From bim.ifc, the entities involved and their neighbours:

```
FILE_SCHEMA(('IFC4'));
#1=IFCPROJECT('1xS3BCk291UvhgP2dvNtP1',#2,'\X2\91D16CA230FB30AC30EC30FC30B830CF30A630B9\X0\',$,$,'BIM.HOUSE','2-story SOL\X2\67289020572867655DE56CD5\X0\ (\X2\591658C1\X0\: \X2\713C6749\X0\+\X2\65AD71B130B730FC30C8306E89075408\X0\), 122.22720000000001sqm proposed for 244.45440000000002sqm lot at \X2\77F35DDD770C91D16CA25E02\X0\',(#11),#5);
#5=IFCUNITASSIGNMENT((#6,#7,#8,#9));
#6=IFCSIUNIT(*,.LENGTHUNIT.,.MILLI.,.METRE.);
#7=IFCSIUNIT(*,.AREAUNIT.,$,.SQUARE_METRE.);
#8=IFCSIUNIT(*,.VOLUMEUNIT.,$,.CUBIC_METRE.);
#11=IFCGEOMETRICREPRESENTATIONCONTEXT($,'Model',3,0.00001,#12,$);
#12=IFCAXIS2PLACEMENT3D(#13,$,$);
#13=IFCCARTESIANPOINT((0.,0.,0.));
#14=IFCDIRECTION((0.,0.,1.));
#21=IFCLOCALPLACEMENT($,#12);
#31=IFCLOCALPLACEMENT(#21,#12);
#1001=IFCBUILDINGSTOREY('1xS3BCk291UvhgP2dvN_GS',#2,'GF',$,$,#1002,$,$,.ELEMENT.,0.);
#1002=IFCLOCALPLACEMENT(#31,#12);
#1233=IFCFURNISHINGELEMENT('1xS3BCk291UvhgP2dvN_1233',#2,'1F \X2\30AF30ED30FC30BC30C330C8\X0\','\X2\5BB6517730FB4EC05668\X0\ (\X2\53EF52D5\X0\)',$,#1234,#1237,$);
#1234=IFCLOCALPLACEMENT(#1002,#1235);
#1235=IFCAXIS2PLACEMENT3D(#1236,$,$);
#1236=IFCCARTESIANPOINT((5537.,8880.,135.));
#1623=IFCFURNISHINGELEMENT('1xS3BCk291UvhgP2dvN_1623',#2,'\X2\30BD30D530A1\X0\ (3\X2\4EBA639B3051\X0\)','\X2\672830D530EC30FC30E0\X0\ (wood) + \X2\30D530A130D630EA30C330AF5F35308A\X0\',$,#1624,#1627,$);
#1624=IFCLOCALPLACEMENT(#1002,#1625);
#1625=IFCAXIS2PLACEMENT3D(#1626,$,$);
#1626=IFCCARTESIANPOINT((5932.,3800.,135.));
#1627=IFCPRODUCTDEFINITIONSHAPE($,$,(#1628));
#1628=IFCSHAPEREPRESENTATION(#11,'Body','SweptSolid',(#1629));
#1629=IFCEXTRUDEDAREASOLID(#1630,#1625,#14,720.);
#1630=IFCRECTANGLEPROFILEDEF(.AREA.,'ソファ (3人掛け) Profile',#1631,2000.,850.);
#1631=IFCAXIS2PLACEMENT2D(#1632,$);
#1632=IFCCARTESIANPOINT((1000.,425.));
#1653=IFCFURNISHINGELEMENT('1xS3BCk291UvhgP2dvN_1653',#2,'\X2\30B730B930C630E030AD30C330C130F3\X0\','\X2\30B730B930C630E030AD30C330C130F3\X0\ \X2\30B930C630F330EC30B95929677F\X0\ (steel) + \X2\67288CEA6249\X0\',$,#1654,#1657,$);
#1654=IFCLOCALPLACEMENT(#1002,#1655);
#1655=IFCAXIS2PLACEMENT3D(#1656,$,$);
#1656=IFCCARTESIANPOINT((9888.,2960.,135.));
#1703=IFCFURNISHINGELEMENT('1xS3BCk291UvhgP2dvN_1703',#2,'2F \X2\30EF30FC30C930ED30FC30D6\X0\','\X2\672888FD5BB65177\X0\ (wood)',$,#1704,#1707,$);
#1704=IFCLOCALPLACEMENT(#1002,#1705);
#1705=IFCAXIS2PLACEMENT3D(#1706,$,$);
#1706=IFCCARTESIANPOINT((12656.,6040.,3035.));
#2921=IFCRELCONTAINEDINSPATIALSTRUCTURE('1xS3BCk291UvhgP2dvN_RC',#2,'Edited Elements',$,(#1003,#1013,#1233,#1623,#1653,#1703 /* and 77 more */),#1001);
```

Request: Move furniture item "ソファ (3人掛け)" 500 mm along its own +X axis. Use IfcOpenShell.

```python
import ifcopenshell
import ifcopenshell.api.geometry
import ifcopenshell.util.placement

model = ifcopenshell.open("bim.ifc")

item = model.by_guid("1xS3BCk291UvhgP2dvN_1623")
matrix = ifcopenshell.util.placement.get_local_placement(item.ObjectPlacement)
matrix[:3, 3] += matrix[:3, 0] * 500.0
ifcopenshell.api.geometry.edit_object_placement(model, product=item, matrix=matrix, is_si=False)

print(ifcopenshell.util.placement.get_local_placement(item.ObjectPlacement).round(3) + 0.0)

model.write("bim_v2.ifc")
```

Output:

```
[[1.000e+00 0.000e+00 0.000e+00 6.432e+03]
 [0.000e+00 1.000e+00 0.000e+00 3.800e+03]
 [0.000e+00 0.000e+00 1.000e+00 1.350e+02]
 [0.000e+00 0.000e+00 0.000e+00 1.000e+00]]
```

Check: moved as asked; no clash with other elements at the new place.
